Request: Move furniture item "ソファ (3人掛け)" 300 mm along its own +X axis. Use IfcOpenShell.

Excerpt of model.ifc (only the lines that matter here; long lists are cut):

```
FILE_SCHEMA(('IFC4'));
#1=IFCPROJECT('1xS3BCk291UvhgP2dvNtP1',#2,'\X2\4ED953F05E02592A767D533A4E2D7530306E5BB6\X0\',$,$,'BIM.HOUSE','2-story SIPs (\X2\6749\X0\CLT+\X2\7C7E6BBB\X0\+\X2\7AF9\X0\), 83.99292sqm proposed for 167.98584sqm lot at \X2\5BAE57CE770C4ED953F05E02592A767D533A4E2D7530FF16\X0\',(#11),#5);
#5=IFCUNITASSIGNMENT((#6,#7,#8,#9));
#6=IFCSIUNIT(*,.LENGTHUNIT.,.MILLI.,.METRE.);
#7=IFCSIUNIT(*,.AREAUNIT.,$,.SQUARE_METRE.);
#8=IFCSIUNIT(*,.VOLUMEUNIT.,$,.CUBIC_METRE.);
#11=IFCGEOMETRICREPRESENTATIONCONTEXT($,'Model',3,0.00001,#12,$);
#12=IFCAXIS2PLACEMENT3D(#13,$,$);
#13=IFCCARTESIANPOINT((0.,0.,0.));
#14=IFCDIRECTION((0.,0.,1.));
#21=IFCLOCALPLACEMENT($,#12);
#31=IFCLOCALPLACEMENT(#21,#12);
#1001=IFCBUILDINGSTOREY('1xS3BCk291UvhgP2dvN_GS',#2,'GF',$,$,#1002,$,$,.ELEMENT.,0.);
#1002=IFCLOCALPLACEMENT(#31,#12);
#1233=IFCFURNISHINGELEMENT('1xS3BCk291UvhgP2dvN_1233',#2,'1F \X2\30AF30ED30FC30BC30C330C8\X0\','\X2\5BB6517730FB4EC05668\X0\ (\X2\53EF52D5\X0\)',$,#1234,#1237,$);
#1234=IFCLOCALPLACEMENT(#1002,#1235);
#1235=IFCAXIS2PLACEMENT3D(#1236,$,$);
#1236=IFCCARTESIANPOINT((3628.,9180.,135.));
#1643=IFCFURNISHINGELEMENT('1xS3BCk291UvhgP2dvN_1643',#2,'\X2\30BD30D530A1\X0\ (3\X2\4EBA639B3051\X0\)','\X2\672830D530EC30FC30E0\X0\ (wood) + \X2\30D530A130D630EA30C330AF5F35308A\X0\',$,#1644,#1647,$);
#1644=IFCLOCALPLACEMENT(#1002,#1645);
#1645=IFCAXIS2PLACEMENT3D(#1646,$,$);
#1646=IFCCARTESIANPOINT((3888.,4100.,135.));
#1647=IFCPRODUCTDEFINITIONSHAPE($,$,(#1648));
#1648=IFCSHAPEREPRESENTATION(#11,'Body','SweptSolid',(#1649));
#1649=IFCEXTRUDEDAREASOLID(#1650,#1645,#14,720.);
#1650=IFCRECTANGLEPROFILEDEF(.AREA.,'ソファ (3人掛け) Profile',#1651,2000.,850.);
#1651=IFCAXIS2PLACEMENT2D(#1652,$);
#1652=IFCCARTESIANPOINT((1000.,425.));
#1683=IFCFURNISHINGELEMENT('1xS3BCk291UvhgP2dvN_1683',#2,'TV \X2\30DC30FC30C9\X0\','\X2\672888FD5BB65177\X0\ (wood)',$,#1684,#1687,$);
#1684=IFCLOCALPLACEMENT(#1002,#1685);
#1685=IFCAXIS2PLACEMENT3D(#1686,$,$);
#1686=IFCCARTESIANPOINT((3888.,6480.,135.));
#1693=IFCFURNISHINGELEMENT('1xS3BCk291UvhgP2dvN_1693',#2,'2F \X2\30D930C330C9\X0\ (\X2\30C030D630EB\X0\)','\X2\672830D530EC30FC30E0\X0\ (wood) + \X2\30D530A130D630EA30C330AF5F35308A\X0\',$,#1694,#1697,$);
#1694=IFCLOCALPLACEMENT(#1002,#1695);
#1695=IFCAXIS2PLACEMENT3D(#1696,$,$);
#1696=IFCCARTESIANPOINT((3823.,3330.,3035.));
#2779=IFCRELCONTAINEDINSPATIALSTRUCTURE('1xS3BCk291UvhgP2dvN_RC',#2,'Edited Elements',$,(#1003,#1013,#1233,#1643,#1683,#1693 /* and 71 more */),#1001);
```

```python
import ifcopenshell
import ifcopenshell.api.geometry
import ifcopenshell.util.placement
import ifcopenshell.util.unit

model = ifcopenshell.open("model.ifc")
unit_scale = ifcopenshell.util.unit.calculate_unit_scale(model)

item = model.by_guid("1xS3BCk291UvhgP2dvN_1643")
matrix = ifcopenshell.util.placement.get_local_placement(item.ObjectPlacement)
matrix[:3, 3] += matrix[:3, 0] * 0.3 / unit_scale
ifcopenshell.api.geometry.edit_object_placement(model, product=item, matrix=matrix, is_si=False)

print(ifcopenshell.util.placement.get_local_placement(item.ObjectPlacement).round(3) + 0.0)

model.write("model_updated.ifc")
```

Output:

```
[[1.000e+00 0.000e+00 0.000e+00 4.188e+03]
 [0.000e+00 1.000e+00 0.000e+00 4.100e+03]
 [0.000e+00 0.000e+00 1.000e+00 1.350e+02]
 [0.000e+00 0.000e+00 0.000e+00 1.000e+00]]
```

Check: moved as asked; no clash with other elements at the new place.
